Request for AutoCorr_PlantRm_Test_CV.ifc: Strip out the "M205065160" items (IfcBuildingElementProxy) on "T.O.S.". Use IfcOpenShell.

First a look at what the model holds.

```python
import ifcopenshell
import ifcopenshell.util.element

model = ifcopenshell.open("AutoCorr_PlantRm_Test_CV.ifc")
print(model.schema)
storey = next(s for s in model.by_type("IfcBuildingStorey") if s.Name == "T.O.S.")
proxies = [e for e in ifcopenshell.util.element.get_decomposition(storey) if e.is_a("IfcBuildingElementProxy")]
seen = {}
for e in proxies:
    element_type = ifcopenshell.util.element.get_type(e)
    name = element_type.Name if element_type not in (None, e) else None
    seen[name] = seen.get(name, 0) + 1
for name, count in sorted(seen.items(), key=str):
    print(count, "x", name)
```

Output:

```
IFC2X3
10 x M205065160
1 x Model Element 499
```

```python
import ifcopenshell
import ifcopenshell.api.root
import ifcopenshell.util.element

model = ifcopenshell.open("AutoCorr_PlantRm_Test_CV.ifc")

storey = next(s for s in model.by_type("IfcBuildingStorey") if s.Name == "T.O.S.")
proxies = [e for e in ifcopenshell.util.element.get_decomposition(storey) if e.is_a("IfcBuildingElementProxy")]
targets = [e for e in proxies if (t := ifcopenshell.util.element.get_type(e)) not in (None, e) and t.Name == "M205065160"]

for e in targets:
    ifcopenshell.api.root.remove_product(model, product=e)
print(len(targets), "removed")

model.write("AutoCorr_PlantRm_Test_CV_rev.ifc")
```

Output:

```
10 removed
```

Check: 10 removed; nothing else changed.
